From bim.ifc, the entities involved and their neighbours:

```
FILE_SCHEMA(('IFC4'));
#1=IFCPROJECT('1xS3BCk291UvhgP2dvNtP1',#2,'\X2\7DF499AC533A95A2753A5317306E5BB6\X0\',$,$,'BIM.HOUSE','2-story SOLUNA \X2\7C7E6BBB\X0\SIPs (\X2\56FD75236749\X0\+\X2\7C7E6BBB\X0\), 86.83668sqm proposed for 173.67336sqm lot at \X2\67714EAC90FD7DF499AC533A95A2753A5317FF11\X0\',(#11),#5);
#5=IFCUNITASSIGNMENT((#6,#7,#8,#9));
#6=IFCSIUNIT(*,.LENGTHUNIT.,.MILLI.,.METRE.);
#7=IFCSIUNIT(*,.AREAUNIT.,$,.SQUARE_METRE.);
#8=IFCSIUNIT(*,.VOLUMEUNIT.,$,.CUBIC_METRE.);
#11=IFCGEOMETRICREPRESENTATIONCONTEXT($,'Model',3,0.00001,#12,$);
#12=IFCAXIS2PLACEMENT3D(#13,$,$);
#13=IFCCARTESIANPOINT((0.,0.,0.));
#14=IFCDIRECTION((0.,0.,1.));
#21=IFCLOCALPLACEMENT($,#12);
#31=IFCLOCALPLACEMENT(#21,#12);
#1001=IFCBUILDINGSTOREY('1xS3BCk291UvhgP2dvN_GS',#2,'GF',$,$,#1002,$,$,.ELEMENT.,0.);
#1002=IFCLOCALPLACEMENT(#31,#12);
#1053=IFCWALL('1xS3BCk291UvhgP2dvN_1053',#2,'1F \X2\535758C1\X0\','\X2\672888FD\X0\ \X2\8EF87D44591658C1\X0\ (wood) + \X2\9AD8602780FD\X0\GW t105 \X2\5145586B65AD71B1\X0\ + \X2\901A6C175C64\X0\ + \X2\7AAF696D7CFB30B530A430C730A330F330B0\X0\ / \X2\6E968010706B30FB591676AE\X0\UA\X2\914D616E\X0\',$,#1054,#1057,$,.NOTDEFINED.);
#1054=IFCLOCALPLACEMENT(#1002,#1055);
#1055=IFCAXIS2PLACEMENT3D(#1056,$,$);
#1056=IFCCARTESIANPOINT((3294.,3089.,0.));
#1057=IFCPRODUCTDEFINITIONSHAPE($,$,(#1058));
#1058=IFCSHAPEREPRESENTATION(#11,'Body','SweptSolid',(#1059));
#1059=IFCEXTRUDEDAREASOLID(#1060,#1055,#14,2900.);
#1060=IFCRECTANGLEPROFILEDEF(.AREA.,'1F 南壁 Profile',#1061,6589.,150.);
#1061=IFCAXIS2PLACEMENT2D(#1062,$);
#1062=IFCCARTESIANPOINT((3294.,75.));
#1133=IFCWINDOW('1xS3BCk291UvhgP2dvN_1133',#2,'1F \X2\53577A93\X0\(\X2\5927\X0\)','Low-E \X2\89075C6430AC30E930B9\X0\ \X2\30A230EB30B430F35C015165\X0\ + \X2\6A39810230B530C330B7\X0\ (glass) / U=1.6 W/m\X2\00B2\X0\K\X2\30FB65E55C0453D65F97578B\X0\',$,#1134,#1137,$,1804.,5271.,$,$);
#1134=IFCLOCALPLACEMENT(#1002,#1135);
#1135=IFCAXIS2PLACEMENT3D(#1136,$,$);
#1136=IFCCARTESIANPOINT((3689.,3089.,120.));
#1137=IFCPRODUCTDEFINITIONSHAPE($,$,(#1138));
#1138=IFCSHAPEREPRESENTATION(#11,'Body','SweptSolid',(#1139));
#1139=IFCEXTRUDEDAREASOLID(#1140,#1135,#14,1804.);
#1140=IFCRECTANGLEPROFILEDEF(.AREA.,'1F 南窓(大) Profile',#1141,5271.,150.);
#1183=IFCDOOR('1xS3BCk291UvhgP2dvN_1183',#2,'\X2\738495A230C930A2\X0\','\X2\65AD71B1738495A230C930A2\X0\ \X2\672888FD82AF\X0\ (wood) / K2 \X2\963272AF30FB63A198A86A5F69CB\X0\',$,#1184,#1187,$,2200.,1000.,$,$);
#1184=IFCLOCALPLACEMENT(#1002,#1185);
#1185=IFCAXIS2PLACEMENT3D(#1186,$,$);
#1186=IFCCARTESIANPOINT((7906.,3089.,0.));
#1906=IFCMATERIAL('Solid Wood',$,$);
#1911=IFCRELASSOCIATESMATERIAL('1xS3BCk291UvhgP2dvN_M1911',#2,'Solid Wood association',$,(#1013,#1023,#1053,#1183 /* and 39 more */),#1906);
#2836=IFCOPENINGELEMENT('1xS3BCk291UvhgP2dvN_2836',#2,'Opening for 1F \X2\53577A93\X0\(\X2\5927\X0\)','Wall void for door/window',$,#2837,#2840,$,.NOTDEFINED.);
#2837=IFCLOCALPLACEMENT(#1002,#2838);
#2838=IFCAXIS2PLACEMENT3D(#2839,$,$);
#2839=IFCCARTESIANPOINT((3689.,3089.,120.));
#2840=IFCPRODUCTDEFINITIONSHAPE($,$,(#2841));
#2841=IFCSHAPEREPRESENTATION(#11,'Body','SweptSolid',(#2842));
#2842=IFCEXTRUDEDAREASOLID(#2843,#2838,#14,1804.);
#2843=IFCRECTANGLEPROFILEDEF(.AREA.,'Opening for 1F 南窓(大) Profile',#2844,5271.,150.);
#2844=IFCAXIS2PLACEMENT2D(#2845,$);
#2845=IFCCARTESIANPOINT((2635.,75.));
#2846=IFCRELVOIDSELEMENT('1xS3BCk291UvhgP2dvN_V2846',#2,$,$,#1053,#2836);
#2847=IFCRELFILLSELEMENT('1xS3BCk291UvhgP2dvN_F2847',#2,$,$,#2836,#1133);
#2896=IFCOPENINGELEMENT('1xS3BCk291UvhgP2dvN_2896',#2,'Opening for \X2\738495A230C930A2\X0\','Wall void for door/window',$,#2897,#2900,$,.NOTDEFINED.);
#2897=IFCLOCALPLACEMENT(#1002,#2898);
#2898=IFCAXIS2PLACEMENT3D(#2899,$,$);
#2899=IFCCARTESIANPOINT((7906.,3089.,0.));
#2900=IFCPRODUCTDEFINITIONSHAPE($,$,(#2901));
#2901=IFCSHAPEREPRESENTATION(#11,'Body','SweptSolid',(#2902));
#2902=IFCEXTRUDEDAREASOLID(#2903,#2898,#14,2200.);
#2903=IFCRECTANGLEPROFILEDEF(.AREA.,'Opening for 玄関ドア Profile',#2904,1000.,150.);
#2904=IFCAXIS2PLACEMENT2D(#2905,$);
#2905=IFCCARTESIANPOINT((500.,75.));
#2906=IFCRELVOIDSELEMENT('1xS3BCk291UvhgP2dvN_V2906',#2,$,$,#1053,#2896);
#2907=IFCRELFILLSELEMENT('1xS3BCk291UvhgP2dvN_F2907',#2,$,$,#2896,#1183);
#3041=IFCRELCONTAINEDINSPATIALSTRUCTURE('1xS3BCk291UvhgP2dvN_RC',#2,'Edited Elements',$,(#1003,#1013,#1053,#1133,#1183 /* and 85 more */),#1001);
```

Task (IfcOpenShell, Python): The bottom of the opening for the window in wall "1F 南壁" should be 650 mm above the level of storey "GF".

```python
import numpy as np
import ifcopenshell
import ifcopenshell.api.geometry
import ifcopenshell.geom
import ifcopenshell.util.element
import ifcopenshell.util.placement
import ifcopenshell.util.shape
import ifcopenshell.util.unit

model = ifcopenshell.open("bim.ifc")
unit_scale = ifcopenshell.util.unit.calculate_unit_scale(model)

window = model.by_id(1133)
opening = window.FillsVoids[0].RelatingOpeningElement
storey = ifcopenshell.util.element.get_container(window, ifc_class="IfcBuildingStorey")
level = ifcopenshell.util.placement.get_local_placement(storey.ObjectPlacement)[2, 3]

# The opening's origin need not be at the sill, so measure its lowest point.
shape = ifcopenshell.geom.create_shape(ifcopenshell.geom.settings(), opening)
bottom = ifcopenshell.util.shape.get_shape_bottom_elevation(shape, shape.geometry) / unit_scale
dz = level + 650.0 - bottom

shift = np.array([0.0, 0.0, dz])
# The window is not placed relative to its opening, so move both.
for product in (opening, window):
    matrix = ifcopenshell.util.placement.get_local_placement(product.ObjectPlacement)
    matrix[:3, 3] += shift
    ifcopenshell.api.geometry.edit_object_placement(model, product=product, matrix=matrix, is_si=False)

print(f"moved by {dz * unit_scale:+.3f} m")

model.write("bim_v2.ifc")
```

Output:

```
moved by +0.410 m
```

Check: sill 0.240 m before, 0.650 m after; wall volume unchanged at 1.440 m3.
